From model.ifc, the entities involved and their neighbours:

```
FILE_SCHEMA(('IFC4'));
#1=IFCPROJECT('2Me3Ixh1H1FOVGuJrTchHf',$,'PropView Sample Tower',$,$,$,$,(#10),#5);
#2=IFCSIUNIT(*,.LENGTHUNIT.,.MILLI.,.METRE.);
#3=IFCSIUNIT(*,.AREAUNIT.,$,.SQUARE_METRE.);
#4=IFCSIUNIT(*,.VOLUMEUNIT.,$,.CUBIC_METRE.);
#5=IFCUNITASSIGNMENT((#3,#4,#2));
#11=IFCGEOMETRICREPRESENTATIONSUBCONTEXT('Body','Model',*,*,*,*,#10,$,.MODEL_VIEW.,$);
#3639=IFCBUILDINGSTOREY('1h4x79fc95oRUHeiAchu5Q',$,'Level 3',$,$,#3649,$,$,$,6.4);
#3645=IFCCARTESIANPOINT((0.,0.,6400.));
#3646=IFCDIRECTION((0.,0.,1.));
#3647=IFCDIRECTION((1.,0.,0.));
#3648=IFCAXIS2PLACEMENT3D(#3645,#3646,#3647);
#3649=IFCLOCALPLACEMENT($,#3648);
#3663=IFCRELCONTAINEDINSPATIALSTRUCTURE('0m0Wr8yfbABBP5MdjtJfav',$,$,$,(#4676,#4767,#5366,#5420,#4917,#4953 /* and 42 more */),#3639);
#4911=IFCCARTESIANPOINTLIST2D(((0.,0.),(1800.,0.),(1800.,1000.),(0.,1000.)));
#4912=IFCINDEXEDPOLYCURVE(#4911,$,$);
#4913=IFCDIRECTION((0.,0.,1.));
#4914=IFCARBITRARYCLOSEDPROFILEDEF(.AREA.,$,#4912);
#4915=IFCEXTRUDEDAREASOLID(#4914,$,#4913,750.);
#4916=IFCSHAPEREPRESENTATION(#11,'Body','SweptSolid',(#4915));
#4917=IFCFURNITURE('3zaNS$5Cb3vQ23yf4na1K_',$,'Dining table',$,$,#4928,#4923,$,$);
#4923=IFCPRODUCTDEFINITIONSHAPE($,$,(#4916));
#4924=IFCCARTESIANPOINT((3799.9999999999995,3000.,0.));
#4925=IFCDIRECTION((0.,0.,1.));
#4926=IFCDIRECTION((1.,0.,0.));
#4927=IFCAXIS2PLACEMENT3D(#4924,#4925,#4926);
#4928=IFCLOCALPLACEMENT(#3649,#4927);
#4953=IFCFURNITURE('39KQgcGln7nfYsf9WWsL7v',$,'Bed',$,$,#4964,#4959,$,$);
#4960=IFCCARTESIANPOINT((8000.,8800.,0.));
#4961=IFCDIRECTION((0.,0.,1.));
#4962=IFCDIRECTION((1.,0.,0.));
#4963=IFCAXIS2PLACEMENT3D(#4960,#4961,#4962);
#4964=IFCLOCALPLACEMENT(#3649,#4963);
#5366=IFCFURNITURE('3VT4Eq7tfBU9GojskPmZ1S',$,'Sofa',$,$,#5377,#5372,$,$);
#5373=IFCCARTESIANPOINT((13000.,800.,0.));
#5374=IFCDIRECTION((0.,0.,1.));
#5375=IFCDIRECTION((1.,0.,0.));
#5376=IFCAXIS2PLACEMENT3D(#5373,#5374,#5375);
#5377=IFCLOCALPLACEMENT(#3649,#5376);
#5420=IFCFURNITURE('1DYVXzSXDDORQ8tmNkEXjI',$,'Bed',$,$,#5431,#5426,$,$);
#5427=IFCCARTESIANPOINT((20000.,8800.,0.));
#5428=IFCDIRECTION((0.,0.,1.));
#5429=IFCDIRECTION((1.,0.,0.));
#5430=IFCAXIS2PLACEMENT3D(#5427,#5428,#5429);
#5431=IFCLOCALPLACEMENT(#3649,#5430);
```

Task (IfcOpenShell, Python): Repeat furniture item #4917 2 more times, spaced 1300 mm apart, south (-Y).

```python
import numpy as np
import ifcopenshell
import ifcopenshell.api.geometry
import ifcopenshell.api.root
import ifcopenshell.util.element
import ifcopenshell.util.placement
import ifcopenshell.util.unit

model = ifcopenshell.open("model.ifc")
unit_scale = ifcopenshell.util.unit.calculate_unit_scale(model)

source = model.by_guid("3zaNS$5Cb3vQ23yf4na1K_")
base = ifcopenshell.util.placement.get_local_placement(source.ObjectPlacement)
step = np.array([0.0, -1.0, 0.0]) * 1.3 / unit_scale

for i in range(1, 3):
    copy = ifcopenshell.api.root.copy_class(model, product=source)
    copy.Representation = ifcopenshell.util.element.copy_deep(
        model, source.Representation, exclude=["IfcGeometricRepresentationContext", "IfcRepresentationMap"]
    )
    matrix = base.copy()
    matrix[:3, 3] += i * step
    print("added at", matrix[:3, 3].round(3) + 0.0)
    ifcopenshell.api.geometry.edit_object_placement(model, product=copy, matrix=matrix, is_si=False)

model.write("model_rev.ifc")
```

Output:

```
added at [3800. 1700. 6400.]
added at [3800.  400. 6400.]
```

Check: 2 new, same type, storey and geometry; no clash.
